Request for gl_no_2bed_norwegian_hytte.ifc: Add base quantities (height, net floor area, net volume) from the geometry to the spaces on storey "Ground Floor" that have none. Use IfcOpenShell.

First a look at what the model holds.

```python
import ifcopenshell
import ifcopenshell.util.element
import ifcopenshell.util.unit

model = ifcopenshell.open("gl_no_2bed_norwegian_hytte.ifc")
print(model.schema)
for unit_type in ("LENGTHUNIT", "AREAUNIT", "VOLUMEUNIT"):
    print(unit_type, ifcopenshell.util.unit.calculate_unit_scale(model, unit_type))
storey = next(s for s in model.by_type("IfcBuildingStorey") if s.Name == "Ground Floor")
spaces = [e for e in ifcopenshell.util.element.get_decomposition(storey) if e.is_a("IfcSpace")]
for e in sorted(spaces, key=lambda e: e.id()):
    print(e.id(), e.is_a(), e.Name, list(ifcopenshell.util.element.get_psets(e, qtos_only=True)), sep=" | ")
```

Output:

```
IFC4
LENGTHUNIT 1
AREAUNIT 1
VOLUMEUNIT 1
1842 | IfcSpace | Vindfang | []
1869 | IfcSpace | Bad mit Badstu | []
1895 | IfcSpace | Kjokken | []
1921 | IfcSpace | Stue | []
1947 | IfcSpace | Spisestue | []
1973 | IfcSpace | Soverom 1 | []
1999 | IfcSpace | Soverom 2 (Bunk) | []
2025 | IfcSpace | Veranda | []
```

```python
import ifcopenshell
import ifcopenshell.api.pset
import ifcopenshell.geom
import ifcopenshell.util.element
import ifcopenshell.util.shape
import ifcopenshell.util.unit

model = ifcopenshell.open("gl_no_2bed_norwegian_hytte.ifc")
unit_scale = ifcopenshell.util.unit.calculate_unit_scale(model)
area_scale = ifcopenshell.util.unit.calculate_unit_scale(model, "AREAUNIT")
volume_scale = ifcopenshell.util.unit.calculate_unit_scale(model, "VOLUMEUNIT")
settings = ifcopenshell.geom.settings()

storey = next(s for s in model.by_type("IfcBuildingStorey") if s.Name == "Ground Floor")
spaces = [e for e in ifcopenshell.util.element.get_decomposition(storey) if e.is_a("IfcSpace")]

for e in sorted(spaces, key=lambda e: e.id()):
    if ifcopenshell.util.element.get_psets(e, qtos_only=True, should_inherit=False):
        continue
    # Geometry comes back in metres, in the element's own axes.
    shape = ifcopenshell.geom.create_shape(settings, e)
    values = {
        "Height": ifcopenshell.util.shape.get_z(shape.geometry) / unit_scale,
        "NetFloorArea": ifcopenshell.util.shape.get_footprint_area(shape.geometry) / area_scale,
        "NetVolume": ifcopenshell.util.shape.get_volume(shape.geometry) / volume_scale,
    }
    qto = ifcopenshell.api.pset.add_qto(model, product=e, name="Qto_SpaceBaseQuantities")
    ifcopenshell.api.pset.edit_qto(model, qto=qto, properties=values)
    print(e.id(), {k: round(v, 3) for k, v in values.items()})

model.write("gl_no_2bed_norwegian_hytte_rev.ifc")
```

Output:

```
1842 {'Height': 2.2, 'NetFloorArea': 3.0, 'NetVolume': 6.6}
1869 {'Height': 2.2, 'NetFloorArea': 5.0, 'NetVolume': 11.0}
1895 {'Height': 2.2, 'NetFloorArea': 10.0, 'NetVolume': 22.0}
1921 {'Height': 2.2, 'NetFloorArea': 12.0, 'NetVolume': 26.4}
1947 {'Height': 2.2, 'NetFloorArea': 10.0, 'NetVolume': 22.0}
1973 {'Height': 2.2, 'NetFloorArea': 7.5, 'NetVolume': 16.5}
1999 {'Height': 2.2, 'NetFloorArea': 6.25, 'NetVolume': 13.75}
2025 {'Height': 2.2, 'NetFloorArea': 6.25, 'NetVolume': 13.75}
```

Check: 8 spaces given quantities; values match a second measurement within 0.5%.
